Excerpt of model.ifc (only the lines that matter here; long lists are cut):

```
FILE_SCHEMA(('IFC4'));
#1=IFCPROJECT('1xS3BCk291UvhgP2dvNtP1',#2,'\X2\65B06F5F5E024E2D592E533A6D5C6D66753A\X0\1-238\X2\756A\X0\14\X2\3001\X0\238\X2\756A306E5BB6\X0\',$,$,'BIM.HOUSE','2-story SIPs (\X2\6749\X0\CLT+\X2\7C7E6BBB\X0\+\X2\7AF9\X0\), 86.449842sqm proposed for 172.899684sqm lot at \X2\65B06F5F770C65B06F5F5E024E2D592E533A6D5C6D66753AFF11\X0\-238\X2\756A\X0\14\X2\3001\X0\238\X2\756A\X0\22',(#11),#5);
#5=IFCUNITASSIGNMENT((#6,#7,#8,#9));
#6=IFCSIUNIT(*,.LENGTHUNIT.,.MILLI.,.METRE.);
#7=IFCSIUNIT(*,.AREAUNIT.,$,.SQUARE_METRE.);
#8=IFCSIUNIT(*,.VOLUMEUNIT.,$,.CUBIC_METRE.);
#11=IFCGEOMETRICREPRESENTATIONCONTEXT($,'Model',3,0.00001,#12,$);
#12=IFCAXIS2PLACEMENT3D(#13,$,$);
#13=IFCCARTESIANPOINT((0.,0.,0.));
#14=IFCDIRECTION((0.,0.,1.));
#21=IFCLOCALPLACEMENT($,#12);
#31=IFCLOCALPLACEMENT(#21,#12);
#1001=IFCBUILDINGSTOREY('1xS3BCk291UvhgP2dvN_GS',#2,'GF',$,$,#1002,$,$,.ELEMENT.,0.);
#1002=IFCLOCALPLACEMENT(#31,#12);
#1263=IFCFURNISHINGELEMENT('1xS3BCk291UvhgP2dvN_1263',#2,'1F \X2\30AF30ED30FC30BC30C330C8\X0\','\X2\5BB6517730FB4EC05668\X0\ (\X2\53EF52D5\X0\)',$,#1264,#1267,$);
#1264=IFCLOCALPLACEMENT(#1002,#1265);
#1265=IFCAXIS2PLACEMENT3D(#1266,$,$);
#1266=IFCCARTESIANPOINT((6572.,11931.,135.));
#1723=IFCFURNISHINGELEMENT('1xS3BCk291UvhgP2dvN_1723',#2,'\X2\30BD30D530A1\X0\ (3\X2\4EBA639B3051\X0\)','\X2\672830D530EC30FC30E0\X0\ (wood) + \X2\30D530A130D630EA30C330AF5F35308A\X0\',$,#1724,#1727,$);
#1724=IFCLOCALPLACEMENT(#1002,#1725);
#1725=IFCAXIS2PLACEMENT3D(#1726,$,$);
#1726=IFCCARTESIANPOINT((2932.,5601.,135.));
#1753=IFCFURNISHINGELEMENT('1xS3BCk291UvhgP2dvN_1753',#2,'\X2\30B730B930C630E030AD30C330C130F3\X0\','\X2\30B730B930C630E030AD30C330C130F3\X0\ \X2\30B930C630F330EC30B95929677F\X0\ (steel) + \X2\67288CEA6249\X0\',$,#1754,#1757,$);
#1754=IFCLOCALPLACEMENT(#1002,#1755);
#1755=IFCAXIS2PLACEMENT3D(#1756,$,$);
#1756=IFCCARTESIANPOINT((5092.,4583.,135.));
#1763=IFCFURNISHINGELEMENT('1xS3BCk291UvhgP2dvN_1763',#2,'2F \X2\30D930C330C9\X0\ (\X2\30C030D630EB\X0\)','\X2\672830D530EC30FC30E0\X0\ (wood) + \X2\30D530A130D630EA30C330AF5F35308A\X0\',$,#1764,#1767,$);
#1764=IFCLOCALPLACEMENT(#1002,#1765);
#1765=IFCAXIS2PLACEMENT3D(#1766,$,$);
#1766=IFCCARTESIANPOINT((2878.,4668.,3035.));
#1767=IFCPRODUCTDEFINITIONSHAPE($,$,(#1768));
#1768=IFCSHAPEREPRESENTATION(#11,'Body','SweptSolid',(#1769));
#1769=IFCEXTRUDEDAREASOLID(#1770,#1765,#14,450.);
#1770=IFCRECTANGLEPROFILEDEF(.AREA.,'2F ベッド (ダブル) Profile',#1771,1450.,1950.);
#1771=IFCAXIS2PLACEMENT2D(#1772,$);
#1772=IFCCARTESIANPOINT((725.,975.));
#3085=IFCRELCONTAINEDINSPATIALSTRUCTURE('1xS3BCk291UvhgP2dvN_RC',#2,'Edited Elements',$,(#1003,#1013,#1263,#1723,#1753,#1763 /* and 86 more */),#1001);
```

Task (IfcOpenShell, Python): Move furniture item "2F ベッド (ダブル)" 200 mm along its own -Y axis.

```python
import ifcopenshell
import ifcopenshell.api.geometry
import ifcopenshell.util.placement
import ifcopenshell.util.unit

model = ifcopenshell.open("model.ifc")
unit_scale = ifcopenshell.util.unit.calculate_unit_scale(model)

item = model.by_guid("1xS3BCk291UvhgP2dvN_1763")
matrix = ifcopenshell.util.placement.get_local_placement(item.ObjectPlacement)
matrix[:3, 3] -= matrix[:3, 1] * 0.2 / unit_scale
ifcopenshell.api.geometry.edit_object_placement(model, product=item, matrix=matrix, is_si=False)

print(ifcopenshell.util.placement.get_local_placement(item.ObjectPlacement).round(3) + 0.0)

model.write("model_v2.ifc")
```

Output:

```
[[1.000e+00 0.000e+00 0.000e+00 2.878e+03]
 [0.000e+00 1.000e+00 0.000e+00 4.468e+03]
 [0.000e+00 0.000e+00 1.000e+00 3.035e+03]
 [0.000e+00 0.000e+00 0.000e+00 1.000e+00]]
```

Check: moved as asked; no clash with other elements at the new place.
